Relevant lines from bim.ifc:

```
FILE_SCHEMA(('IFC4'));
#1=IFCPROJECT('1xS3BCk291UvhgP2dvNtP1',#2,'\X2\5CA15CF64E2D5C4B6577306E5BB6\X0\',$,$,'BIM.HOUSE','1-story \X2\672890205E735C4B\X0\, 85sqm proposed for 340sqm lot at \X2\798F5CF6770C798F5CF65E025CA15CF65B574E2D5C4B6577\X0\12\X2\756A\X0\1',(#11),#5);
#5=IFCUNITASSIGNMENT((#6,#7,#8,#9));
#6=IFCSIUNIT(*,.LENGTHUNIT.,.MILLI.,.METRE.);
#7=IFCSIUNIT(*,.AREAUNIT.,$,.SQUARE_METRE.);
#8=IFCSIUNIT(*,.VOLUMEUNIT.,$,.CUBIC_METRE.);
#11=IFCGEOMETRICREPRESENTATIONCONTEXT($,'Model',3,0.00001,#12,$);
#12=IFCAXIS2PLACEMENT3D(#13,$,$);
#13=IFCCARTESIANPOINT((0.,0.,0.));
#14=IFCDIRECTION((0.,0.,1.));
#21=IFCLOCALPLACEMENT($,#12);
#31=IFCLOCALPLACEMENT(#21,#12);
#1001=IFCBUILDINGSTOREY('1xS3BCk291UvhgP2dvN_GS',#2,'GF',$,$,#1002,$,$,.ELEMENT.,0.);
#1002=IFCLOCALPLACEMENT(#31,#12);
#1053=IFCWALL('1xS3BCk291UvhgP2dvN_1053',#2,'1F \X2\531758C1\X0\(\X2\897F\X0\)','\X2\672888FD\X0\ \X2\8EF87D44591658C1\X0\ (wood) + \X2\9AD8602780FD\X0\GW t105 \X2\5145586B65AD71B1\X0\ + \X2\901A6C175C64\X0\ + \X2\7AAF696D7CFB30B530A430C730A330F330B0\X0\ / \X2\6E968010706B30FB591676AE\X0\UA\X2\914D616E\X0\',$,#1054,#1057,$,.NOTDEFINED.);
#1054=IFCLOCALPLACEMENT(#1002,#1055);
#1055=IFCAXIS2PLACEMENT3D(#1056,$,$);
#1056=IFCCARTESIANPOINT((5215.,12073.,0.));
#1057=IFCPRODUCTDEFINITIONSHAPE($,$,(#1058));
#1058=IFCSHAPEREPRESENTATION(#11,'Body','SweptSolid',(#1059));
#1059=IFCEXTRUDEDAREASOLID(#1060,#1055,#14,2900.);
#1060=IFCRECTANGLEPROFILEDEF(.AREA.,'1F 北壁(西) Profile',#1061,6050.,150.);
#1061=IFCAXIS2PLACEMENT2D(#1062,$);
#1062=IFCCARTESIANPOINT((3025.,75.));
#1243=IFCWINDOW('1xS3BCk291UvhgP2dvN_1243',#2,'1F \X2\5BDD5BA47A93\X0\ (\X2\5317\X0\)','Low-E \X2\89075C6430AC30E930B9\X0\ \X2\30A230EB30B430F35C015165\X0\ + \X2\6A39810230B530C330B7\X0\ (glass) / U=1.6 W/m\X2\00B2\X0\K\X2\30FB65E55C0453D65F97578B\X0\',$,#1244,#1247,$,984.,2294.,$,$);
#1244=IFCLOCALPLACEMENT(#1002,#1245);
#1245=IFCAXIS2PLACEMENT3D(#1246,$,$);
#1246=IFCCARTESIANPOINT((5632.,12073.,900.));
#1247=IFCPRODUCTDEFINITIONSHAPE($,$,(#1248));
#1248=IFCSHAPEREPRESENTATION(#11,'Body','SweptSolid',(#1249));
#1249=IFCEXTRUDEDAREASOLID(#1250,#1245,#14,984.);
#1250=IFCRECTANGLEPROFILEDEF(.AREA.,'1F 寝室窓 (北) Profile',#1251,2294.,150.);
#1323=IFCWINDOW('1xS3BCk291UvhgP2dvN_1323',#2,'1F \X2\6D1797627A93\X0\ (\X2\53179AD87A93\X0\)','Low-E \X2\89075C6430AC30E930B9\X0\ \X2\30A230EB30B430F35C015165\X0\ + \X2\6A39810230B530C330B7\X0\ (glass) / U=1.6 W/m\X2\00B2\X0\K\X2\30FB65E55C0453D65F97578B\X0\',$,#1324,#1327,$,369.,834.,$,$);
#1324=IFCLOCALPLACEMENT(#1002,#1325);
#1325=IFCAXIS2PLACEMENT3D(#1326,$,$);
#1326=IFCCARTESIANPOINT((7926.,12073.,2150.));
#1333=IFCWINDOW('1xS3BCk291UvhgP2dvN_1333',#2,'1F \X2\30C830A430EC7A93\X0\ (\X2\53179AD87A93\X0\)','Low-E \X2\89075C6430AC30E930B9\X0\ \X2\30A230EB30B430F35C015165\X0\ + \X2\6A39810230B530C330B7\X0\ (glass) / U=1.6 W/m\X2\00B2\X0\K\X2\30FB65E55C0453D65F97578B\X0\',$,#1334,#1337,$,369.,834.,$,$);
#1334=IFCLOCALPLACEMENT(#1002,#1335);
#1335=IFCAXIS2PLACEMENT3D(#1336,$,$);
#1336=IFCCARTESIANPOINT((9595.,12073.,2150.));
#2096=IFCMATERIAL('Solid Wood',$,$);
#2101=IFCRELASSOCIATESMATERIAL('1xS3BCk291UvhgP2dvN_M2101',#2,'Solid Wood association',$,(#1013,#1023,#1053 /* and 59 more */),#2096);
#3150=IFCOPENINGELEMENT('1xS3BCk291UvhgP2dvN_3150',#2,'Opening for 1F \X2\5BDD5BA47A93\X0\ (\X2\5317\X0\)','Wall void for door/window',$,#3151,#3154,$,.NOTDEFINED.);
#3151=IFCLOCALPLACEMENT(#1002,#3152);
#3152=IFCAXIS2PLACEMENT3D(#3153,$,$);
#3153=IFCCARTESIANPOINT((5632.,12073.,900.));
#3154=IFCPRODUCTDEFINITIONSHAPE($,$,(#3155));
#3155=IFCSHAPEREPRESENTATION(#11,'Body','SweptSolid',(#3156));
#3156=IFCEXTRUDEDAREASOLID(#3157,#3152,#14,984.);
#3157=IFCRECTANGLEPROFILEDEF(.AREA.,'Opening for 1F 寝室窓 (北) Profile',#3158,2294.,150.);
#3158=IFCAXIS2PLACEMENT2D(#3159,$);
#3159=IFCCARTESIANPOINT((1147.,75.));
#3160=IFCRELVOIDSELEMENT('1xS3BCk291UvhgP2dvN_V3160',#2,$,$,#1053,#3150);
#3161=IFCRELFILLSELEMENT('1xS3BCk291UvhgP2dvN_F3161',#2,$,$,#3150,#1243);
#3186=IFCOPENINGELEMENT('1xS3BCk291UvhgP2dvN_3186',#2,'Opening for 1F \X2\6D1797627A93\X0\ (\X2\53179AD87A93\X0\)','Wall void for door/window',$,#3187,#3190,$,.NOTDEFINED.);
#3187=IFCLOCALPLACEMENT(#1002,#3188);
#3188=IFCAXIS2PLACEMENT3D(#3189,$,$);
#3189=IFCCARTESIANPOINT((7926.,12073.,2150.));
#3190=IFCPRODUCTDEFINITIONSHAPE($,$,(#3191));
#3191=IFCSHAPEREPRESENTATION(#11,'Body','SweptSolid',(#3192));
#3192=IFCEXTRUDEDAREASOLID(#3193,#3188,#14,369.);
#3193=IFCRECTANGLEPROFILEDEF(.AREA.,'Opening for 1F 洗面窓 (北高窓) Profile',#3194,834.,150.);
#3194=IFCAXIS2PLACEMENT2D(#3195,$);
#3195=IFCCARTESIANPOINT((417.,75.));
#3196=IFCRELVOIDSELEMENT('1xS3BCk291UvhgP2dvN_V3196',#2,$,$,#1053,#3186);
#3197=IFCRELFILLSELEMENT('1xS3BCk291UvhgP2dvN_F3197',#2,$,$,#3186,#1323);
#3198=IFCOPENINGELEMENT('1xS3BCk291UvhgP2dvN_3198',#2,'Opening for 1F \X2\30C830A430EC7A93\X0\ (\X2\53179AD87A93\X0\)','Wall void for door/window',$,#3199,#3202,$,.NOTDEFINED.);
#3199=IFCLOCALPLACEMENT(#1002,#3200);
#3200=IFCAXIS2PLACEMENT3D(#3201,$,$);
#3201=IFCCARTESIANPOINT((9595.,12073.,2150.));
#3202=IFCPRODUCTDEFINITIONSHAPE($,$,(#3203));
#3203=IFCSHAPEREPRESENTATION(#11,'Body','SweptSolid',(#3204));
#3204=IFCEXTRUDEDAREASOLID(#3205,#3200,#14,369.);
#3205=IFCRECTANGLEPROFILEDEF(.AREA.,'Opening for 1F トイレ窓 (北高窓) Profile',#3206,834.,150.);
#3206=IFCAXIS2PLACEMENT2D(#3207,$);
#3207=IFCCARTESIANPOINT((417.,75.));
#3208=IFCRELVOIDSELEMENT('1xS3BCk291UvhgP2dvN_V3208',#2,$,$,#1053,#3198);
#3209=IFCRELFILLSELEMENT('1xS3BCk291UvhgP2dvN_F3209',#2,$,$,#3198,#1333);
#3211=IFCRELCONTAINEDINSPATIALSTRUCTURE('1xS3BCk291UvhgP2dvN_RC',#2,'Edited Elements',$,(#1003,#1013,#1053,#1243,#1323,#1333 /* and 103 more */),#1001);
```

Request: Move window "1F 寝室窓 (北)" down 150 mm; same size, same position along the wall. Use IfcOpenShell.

```python
import numpy as np
import ifcopenshell
import ifcopenshell.api.geometry
import ifcopenshell.util.placement
import ifcopenshell.util.unit

model = ifcopenshell.open("bim.ifc")
unit_scale = ifcopenshell.util.unit.calculate_unit_scale(model)

window = model.by_guid("1xS3BCk291UvhgP2dvN_1243")
opening = window.FillsVoids[0].RelatingOpeningElement
dz = -0.15 / unit_scale

shift = np.array([0.0, 0.0, dz])
# The window is not placed relative to its opening, so move both.
for product in (opening, window):
    matrix = ifcopenshell.util.placement.get_local_placement(product.ObjectPlacement)
    matrix[:3, 3] += shift
    ifcopenshell.api.geometry.edit_object_placement(model, product=product, matrix=matrix, is_si=False)

print(f"moved by {dz * unit_scale:+.3f} m")

model.write("bim_updated.ifc")
```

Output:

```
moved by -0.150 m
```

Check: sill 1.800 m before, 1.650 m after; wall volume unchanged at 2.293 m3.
